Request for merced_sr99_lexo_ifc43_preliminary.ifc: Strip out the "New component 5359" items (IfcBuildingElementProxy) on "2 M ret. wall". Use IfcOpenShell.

First a look at what the model holds.

```python
import ifcopenshell
import ifcopenshell.util.element

model = ifcopenshell.open("merced_sr99_lexo_ifc43_preliminary.ifc")
print(model.schema)
storey = next(s for s in model.by_type("IfcBuildingStorey") if s.Name == "2 M ret. wall")
proxies = [e for e in ifcopenshell.util.element.get_decomposition(storey) if e.is_a("IfcBuildingElementProxy")]
seen = {}
for e in proxies:
    element_type = ifcopenshell.util.element.get_type(e)
    name = element_type.Name if element_type not in (None, e) else None
    seen[name] = seen.get(name, 0) + 1
for name, count in sorted(seen.items(), key=str):
    print(count, "x", name)
```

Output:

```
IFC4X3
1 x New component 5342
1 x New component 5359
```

```python
import ifcopenshell
import ifcopenshell.api.root
import ifcopenshell.util.element

model = ifcopenshell.open("merced_sr99_lexo_ifc43_preliminary.ifc")

storey = next(s for s in model.by_type("IfcBuildingStorey") if s.Name == "2 M ret. wall")
proxies = [e for e in ifcopenshell.util.element.get_decomposition(storey) if e.is_a("IfcBuildingElementProxy")]
targets = [e for e in proxies if (t := ifcopenshell.util.element.get_type(e)) not in (None, e) and t.Name == "New component 5359"]

for e in targets:
    ifcopenshell.api.root.remove_product(model, product=e)
print(len(targets), "removed")

model.write("merced_sr99_lexo_ifc43_preliminary_rev.ifc")
```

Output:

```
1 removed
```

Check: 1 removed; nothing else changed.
